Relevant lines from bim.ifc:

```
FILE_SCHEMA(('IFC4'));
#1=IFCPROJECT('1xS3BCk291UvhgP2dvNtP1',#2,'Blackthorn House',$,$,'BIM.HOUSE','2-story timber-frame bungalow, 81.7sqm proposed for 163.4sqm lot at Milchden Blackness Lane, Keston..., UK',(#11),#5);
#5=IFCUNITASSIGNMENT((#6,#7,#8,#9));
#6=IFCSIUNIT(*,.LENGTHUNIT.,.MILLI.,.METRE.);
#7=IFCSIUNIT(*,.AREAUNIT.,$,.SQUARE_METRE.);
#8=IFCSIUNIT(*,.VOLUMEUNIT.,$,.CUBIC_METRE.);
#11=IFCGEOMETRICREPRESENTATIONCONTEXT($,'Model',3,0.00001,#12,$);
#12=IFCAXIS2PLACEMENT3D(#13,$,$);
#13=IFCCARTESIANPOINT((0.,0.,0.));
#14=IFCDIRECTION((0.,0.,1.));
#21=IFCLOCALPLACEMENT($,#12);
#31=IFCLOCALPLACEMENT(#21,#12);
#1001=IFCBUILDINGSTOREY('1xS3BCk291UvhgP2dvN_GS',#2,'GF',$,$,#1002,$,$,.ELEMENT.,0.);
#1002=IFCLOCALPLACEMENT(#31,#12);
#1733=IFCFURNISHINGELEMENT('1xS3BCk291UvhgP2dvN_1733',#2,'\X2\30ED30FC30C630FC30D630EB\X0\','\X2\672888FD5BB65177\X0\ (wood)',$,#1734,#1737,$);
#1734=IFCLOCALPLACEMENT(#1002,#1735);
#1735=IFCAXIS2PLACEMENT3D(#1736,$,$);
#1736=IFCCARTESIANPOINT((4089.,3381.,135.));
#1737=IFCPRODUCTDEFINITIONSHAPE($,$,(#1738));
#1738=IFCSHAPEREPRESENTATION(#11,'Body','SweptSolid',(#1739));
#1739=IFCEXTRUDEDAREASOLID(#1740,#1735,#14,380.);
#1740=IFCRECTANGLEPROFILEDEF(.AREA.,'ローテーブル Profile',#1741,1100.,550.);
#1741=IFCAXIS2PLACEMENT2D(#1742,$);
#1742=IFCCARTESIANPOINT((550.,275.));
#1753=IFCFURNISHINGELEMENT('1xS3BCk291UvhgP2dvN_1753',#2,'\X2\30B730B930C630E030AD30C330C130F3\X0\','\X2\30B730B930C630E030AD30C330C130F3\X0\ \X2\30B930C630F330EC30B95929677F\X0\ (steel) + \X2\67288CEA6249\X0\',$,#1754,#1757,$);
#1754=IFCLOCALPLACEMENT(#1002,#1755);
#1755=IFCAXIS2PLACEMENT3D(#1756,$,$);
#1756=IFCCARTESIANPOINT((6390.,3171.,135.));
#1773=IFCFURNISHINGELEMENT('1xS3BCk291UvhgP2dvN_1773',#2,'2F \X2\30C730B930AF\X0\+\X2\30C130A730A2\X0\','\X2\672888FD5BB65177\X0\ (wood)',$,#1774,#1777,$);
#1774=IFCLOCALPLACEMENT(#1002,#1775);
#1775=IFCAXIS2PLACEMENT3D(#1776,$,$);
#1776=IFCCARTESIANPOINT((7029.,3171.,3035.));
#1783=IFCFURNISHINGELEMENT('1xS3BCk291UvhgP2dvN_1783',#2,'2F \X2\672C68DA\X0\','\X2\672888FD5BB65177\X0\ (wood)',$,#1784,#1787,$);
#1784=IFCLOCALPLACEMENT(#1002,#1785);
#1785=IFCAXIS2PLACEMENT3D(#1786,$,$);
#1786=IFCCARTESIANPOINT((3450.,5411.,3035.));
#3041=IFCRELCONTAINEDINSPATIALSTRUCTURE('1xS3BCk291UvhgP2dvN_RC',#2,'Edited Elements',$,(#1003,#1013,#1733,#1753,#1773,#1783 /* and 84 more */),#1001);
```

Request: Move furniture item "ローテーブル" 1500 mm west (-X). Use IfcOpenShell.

```python
import ifcopenshell
import ifcopenshell.api.geometry
import ifcopenshell.util.placement

model = ifcopenshell.open("bim.ifc")

item = model.by_guid("1xS3BCk291UvhgP2dvN_1733")
matrix = ifcopenshell.util.placement.get_local_placement(item.ObjectPlacement)
matrix[0, 3] -= 1500.0
ifcopenshell.api.geometry.edit_object_placement(model, product=item, matrix=matrix, is_si=False)

print(ifcopenshell.util.placement.get_local_placement(item.ObjectPlacement).round(3) + 0.0)

model.write("bim_updated.ifc")
```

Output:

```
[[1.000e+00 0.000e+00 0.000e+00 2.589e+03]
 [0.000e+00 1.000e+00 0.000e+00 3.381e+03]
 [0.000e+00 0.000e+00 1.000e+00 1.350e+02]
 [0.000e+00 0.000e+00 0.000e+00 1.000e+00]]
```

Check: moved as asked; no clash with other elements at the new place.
